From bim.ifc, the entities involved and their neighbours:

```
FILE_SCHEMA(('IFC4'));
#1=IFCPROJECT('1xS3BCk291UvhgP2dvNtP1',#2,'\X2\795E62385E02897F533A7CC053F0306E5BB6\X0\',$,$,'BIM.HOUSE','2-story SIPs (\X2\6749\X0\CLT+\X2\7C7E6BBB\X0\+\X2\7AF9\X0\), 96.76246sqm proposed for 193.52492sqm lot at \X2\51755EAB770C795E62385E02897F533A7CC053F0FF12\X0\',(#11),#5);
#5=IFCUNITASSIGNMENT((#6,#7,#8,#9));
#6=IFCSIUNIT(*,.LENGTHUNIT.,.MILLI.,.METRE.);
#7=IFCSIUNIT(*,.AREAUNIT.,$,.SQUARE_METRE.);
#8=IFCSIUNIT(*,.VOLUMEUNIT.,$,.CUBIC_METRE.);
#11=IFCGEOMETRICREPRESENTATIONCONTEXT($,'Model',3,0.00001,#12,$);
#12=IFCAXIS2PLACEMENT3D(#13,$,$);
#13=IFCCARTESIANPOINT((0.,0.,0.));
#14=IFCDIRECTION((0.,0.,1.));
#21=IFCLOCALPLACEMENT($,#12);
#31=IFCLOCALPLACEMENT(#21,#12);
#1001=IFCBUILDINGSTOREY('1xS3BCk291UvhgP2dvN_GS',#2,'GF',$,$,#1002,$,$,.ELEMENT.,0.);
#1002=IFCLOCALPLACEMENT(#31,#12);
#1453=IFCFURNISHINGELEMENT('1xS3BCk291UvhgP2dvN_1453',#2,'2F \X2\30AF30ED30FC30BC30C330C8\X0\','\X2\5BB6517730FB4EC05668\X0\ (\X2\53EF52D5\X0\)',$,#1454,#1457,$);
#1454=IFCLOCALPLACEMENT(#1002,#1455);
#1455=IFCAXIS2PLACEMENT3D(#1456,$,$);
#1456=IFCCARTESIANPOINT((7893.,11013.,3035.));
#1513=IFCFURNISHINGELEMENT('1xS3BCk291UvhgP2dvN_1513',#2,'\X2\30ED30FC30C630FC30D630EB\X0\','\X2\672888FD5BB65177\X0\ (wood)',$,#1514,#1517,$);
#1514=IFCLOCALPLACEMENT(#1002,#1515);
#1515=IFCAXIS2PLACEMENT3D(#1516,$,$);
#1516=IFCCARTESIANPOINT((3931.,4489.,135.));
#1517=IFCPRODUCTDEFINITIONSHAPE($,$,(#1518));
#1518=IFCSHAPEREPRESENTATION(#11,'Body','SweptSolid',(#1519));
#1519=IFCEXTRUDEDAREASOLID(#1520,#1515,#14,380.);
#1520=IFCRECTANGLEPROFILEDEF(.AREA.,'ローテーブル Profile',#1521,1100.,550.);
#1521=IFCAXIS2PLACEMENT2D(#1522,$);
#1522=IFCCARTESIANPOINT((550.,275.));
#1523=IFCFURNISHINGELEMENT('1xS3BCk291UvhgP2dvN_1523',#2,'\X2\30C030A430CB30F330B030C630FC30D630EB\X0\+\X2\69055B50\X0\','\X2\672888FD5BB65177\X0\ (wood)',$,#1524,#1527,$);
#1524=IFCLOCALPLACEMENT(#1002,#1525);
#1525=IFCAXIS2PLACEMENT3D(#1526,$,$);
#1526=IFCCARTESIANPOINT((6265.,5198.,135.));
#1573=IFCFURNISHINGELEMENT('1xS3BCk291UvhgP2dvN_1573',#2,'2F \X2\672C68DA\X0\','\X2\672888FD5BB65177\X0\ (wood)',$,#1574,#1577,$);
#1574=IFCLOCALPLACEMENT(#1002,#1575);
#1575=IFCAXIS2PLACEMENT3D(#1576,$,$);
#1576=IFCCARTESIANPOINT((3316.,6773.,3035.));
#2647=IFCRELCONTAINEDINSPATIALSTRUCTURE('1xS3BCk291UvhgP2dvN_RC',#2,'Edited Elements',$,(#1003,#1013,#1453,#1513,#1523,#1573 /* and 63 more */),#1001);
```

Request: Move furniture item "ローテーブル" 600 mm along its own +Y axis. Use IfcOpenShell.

```python
import ifcopenshell
import ifcopenshell.api.geometry
import ifcopenshell.util.placement
import ifcopenshell.util.unit

model = ifcopenshell.open("bim.ifc")
unit_scale = ifcopenshell.util.unit.calculate_unit_scale(model)

item = model.by_guid("1xS3BCk291UvhgP2dvN_1513")
matrix = ifcopenshell.util.placement.get_local_placement(item.ObjectPlacement)
matrix[:3, 3] += matrix[:3, 1] * 0.6 / unit_scale
ifcopenshell.api.geometry.edit_object_placement(model, product=item, matrix=matrix, is_si=False)

print(ifcopenshell.util.placement.get_local_placement(item.ObjectPlacement).round(3) + 0.0)

model.write("bim_rev.ifc")
```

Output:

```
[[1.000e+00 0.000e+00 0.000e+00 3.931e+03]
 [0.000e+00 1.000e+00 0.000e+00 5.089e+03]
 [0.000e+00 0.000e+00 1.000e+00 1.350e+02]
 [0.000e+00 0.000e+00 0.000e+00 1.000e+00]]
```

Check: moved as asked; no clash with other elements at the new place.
